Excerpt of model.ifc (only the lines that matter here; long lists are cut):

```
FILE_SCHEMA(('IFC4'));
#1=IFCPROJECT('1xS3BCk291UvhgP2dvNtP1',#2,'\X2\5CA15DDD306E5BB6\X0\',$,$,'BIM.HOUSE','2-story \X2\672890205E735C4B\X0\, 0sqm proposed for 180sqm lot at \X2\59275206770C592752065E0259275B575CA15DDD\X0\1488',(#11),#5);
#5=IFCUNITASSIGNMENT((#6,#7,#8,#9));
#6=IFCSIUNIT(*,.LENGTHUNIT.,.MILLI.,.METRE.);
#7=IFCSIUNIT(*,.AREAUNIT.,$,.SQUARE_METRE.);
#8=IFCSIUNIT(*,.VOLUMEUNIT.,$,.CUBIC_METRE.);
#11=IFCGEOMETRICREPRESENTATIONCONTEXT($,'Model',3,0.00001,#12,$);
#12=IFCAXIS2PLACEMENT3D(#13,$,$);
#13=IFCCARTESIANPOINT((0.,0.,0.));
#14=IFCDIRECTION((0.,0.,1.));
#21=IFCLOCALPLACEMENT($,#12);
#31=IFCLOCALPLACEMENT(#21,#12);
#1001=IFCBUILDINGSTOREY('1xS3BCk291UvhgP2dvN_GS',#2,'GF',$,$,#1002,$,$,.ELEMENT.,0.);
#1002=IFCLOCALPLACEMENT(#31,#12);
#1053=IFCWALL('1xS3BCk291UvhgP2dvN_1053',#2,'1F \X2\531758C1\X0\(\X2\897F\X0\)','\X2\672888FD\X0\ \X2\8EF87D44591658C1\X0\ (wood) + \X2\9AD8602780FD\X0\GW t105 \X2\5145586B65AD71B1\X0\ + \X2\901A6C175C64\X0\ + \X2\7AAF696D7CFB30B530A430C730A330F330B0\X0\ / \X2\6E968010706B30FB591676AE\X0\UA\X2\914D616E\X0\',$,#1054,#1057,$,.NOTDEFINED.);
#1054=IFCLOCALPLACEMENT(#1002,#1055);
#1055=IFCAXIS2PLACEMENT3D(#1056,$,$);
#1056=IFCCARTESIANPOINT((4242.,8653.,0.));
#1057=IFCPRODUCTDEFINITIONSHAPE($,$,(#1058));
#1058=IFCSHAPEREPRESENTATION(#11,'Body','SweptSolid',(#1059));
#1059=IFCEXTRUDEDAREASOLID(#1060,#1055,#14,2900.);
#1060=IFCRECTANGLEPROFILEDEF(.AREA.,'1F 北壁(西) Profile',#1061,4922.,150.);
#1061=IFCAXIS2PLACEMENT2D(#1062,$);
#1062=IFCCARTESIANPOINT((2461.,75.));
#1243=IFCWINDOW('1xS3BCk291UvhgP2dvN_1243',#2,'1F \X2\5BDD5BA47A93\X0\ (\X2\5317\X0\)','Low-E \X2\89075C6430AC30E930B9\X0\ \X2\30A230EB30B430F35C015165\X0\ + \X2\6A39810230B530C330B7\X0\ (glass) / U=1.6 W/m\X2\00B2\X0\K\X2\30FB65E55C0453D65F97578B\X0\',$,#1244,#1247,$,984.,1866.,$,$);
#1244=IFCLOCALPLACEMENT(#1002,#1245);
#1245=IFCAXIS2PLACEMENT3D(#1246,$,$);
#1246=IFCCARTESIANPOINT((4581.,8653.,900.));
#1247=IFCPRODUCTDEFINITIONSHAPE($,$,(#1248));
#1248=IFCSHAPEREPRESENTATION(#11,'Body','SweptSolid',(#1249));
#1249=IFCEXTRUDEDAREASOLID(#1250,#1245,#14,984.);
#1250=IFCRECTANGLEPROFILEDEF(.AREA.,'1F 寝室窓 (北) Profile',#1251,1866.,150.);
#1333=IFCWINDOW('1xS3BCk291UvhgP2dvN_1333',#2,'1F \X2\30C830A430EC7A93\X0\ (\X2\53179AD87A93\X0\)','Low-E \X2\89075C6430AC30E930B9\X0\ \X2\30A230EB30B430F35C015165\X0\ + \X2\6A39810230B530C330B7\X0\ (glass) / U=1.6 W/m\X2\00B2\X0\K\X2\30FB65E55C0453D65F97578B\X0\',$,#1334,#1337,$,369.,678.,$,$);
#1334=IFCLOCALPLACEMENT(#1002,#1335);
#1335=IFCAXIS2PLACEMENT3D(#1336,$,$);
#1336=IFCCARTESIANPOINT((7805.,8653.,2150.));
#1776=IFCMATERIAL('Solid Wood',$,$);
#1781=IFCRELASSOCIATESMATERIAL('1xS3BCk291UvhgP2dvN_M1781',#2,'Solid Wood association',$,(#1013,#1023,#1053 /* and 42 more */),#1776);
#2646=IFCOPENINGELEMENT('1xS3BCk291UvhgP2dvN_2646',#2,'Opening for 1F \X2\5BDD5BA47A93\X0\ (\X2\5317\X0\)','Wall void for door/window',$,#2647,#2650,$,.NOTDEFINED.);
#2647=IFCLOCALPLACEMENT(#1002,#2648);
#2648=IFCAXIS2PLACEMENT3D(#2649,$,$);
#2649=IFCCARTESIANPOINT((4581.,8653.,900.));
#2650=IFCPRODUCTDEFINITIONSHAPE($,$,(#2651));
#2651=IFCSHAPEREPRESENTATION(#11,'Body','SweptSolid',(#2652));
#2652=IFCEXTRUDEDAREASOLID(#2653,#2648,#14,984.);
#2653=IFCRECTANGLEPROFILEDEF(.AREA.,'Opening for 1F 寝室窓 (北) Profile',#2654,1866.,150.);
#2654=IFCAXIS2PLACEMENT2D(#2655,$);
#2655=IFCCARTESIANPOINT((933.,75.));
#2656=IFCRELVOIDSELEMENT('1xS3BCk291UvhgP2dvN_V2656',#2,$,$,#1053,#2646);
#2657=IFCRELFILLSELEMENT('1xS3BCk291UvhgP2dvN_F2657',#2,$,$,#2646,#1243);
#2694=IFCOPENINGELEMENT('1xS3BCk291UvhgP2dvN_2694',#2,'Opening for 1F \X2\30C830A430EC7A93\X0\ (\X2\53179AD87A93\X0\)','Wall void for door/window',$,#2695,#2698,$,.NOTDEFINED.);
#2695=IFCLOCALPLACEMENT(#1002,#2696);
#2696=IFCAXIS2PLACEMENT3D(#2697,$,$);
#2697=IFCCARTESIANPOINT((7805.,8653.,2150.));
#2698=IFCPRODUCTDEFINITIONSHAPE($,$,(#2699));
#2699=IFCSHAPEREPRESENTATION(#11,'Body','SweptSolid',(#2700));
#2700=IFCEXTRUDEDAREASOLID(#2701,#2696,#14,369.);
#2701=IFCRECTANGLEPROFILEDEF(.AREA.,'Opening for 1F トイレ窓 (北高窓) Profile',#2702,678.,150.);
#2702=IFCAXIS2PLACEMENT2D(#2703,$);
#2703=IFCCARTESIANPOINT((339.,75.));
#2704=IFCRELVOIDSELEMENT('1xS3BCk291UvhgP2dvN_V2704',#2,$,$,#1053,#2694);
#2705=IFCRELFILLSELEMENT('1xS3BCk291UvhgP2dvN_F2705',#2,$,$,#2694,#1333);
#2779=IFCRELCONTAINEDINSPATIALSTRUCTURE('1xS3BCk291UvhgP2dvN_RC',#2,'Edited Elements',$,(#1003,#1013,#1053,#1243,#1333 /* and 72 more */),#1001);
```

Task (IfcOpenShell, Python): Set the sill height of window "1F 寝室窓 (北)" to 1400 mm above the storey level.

```python
import numpy as np
import ifcopenshell
import ifcopenshell.api.geometry
import ifcopenshell.geom
import ifcopenshell.util.element
import ifcopenshell.util.placement
import ifcopenshell.util.shape
import ifcopenshell.util.unit

model = ifcopenshell.open("model.ifc")
unit_scale = ifcopenshell.util.unit.calculate_unit_scale(model)

window = model.by_id(1243)
opening = window.FillsVoids[0].RelatingOpeningElement
storey = ifcopenshell.util.element.get_container(window, ifc_class="IfcBuildingStorey")
level = ifcopenshell.util.placement.get_local_placement(storey.ObjectPlacement)[2, 3]

# The opening's origin need not be at the sill, so measure its lowest point.
shape = ifcopenshell.geom.create_shape(ifcopenshell.geom.settings(), opening)
bottom = ifcopenshell.util.shape.get_shape_bottom_elevation(shape, shape.geometry) / unit_scale
dz = level + 1.4 / unit_scale - bottom

shift = np.array([0.0, 0.0, dz])
# The window is not placed relative to its opening, so move both.
for product in (opening, window):
    matrix = ifcopenshell.util.placement.get_local_placement(product.ObjectPlacement)
    matrix[:3, 3] += shift
    ifcopenshell.api.geometry.edit_object_placement(model, product=product, matrix=matrix, is_si=False)

print(f"moved by {dz * unit_scale:+.3f} m")

model.write("model_updated.ifc")
```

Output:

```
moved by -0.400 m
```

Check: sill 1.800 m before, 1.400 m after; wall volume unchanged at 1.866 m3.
